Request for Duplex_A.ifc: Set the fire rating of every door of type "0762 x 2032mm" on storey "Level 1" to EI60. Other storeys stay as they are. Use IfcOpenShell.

First a look at what the model holds.

```python
import ifcopenshell
import ifcopenshell.util.element

model = ifcopenshell.open("Duplex_A.ifc")
print(model.schema)
storey = next(s for s in model.by_type("IfcBuildingStorey") if s.Name == "Level 1")
doors = [e for e in ifcopenshell.util.element.get_decomposition(storey) if e.is_a("IfcDoor")]
seen = {}
for e in doors:
    element_type = ifcopenshell.util.element.get_type(e)
    key = (element_type.Name if element_type != e and element_type else None, ifcopenshell.util.element.get_pset(e, "Pset_DoorCommon", "FireRating"))
    seen[key] = seen.get(key, 0) + 1
for (name, value), count in sorted(seen.items(), key=str):
    print(count, "x", name, "|", value)
```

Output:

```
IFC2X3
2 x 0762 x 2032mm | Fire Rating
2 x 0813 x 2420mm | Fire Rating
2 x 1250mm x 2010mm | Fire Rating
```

```python
import ifcopenshell
import ifcopenshell.api.pset
import ifcopenshell.util.element

model = ifcopenshell.open("Duplex_A.ifc")

storey = next(s for s in model.by_type("IfcBuildingStorey") if s.Name == "Level 1")
doors = [e for e in ifcopenshell.util.element.get_decomposition(storey) if e.is_a("IfcDoor")]

count = 0
for e in doors:
    element_type = ifcopenshell.util.element.get_type(e)
    if element_type in (None, e) or element_type.Name != "0762 x 2032mm":
        continue
    # add_pset returns the element's existing set when there is one.
    pset = ifcopenshell.api.pset.add_pset(model, product=e, name="Pset_DoorCommon")
    ifcopenshell.api.pset.edit_pset(model, pset=pset, properties={"FireRating": "EI60"})
    count += 1

print(count, "doors updated")

model.write("Duplex_A_edited.ifc")
```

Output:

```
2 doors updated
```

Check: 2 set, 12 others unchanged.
